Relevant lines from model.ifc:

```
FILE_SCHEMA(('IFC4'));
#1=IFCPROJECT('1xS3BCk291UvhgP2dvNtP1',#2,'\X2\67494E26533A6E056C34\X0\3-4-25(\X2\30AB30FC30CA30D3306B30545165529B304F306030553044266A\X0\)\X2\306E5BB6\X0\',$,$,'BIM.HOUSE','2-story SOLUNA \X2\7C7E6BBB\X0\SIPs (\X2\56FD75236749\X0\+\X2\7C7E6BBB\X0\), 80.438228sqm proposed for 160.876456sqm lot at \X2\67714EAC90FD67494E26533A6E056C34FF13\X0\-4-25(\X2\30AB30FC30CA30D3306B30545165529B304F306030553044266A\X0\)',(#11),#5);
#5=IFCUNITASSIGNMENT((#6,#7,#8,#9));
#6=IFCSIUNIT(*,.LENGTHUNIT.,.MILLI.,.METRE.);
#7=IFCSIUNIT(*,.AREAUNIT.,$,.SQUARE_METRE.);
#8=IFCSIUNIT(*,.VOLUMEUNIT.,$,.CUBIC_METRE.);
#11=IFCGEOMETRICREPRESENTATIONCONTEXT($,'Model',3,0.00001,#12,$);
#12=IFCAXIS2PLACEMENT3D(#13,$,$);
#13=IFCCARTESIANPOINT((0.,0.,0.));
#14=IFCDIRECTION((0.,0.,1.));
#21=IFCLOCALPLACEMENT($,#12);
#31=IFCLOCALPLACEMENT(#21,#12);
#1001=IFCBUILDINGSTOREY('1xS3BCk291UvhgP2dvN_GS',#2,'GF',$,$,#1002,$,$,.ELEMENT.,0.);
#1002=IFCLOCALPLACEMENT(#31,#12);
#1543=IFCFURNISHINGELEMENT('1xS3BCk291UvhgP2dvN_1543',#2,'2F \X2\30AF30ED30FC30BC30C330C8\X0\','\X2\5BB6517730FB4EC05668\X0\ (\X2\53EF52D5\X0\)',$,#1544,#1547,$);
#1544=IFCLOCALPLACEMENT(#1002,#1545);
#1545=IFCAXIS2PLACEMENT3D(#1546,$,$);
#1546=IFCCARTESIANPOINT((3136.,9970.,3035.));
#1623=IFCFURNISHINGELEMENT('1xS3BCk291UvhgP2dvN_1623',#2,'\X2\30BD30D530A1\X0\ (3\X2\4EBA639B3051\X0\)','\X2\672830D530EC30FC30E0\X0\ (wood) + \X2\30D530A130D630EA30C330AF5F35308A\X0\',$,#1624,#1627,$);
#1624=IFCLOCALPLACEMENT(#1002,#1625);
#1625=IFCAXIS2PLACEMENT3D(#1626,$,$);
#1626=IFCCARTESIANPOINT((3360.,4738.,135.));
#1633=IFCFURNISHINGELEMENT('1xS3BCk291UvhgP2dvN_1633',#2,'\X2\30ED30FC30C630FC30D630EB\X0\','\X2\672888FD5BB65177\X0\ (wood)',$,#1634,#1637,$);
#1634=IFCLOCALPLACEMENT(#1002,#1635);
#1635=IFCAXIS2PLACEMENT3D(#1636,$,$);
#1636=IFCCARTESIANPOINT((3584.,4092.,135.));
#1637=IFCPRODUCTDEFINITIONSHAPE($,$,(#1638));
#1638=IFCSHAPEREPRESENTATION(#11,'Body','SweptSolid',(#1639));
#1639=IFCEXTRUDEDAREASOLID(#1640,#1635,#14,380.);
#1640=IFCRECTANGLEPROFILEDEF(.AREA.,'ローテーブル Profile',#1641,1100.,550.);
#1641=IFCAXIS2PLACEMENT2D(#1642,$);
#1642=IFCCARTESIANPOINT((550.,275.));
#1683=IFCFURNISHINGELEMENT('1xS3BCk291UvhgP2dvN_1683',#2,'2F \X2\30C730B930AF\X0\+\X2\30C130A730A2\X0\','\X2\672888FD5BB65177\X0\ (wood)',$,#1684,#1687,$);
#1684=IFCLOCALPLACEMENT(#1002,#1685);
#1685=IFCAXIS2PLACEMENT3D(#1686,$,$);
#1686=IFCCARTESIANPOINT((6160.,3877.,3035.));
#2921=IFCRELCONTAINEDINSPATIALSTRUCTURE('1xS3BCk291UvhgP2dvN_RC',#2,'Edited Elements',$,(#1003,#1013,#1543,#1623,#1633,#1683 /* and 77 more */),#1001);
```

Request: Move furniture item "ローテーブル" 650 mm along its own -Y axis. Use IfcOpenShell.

```python
import ifcopenshell
import ifcopenshell.api.geometry
import ifcopenshell.util.placement

model = ifcopenshell.open("model.ifc")

item = model.by_guid("1xS3BCk291UvhgP2dvN_1633")
matrix = ifcopenshell.util.placement.get_local_placement(item.ObjectPlacement)
matrix[:3, 3] -= matrix[:3, 1] * 650.0
ifcopenshell.api.geometry.edit_object_placement(model, product=item, matrix=matrix, is_si=False)

print(ifcopenshell.util.placement.get_local_placement(item.ObjectPlacement).round(3) + 0.0)

model.write("model-out.ifc")
```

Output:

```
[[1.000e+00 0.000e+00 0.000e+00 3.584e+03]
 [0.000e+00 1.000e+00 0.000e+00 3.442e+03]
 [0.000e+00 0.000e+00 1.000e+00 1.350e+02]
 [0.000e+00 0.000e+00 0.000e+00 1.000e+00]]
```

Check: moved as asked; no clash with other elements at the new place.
